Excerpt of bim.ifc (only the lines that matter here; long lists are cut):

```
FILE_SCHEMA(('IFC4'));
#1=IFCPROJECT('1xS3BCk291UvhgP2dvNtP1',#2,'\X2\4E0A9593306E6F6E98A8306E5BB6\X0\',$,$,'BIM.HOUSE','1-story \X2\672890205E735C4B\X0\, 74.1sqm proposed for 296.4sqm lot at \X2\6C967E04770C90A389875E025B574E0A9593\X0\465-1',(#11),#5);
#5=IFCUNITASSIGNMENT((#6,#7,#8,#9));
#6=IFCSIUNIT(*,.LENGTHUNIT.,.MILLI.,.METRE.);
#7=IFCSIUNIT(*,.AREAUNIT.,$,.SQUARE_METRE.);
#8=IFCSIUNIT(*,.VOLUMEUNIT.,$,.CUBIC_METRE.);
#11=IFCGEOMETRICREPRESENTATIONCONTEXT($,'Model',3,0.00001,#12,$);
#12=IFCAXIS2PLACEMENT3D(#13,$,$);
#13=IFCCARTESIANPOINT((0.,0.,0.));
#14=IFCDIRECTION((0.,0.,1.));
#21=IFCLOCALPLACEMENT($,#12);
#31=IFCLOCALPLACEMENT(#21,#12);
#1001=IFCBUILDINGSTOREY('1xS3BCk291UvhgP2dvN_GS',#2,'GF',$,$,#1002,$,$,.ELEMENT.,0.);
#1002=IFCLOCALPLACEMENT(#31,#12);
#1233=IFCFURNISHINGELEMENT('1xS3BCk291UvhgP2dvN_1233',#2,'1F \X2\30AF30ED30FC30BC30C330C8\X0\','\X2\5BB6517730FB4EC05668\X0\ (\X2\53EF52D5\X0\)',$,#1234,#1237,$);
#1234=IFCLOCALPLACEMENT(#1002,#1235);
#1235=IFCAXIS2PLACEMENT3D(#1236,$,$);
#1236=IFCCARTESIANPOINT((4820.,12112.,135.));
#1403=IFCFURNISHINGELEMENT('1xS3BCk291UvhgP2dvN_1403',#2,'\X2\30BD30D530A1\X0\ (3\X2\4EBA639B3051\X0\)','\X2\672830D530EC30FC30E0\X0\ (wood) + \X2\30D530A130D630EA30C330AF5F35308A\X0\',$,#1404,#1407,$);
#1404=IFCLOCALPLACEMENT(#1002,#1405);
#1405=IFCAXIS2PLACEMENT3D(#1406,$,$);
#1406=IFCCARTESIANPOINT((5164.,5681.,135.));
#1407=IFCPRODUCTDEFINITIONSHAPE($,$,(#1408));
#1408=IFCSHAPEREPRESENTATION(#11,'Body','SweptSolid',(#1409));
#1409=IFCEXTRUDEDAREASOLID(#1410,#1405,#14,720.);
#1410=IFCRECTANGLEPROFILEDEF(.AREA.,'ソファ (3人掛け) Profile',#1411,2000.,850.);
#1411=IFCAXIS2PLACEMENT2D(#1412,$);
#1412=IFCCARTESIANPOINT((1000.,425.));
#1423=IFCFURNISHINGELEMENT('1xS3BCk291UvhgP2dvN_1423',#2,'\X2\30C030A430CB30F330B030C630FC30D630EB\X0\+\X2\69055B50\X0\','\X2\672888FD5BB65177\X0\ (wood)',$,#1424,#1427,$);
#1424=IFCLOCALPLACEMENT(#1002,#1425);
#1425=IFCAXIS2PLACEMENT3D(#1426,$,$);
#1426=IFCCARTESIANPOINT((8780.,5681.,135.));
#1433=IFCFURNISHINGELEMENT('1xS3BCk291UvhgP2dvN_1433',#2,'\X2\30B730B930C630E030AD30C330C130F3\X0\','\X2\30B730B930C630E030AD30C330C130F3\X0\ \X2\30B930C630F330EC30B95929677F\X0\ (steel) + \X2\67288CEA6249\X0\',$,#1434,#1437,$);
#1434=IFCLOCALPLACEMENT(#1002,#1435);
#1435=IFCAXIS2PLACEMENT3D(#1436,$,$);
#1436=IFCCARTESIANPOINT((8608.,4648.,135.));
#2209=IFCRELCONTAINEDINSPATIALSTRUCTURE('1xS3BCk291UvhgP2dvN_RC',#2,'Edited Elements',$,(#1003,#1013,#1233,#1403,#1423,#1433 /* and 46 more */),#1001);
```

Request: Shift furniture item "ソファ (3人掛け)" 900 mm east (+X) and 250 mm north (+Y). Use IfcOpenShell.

```python
import ifcopenshell
import ifcopenshell.api.geometry
import ifcopenshell.util.placement
import ifcopenshell.util.unit

model = ifcopenshell.open("bim.ifc")
unit_scale = ifcopenshell.util.unit.calculate_unit_scale(model)

item = model.by_guid("1xS3BCk291UvhgP2dvN_1403")
matrix = ifcopenshell.util.placement.get_local_placement(item.ObjectPlacement)
matrix[0, 3] += 0.9 / unit_scale
matrix[1, 3] += 0.25 / unit_scale
ifcopenshell.api.geometry.edit_object_placement(model, product=item, matrix=matrix, is_si=False)

print(ifcopenshell.util.placement.get_local_placement(item.ObjectPlacement).round(3) + 0.0)

model.write("bim_edited.ifc")
```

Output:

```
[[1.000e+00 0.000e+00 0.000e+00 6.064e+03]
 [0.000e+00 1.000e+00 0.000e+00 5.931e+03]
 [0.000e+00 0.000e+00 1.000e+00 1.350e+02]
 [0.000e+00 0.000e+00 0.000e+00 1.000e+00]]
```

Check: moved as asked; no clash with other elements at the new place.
